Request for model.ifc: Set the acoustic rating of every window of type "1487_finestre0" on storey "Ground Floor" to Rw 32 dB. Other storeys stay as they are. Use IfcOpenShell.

First a look at what the model holds.

```python
import ifcopenshell
import ifcopenshell.util.element

model = ifcopenshell.open("model.ifc")
print(model.schema)
storey = next(s for s in model.by_type("IfcBuildingStorey") if s.Name == "Ground Floor")
windows = [e for e in ifcopenshell.util.element.get_decomposition(storey) if e.is_a("IfcWindow")]
seen = {}
for e in windows:
    element_type = ifcopenshell.util.element.get_type(e)
    key = (element_type.Name if element_type != e and element_type else None, ifcopenshell.util.element.get_pset(e, "Pset_WindowCommon", "AcousticRating"))
    seen[key] = seen.get(key, 0) + 1
for (name, value), count in sorted(seen.items(), key=str):
    print(count, "x", name, "|", value)
```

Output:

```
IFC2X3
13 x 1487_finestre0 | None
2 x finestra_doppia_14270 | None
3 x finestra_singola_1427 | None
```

```python
import ifcopenshell
import ifcopenshell.api.pset
import ifcopenshell.util.element

model = ifcopenshell.open("model.ifc")

storey = next(s for s in model.by_type("IfcBuildingStorey") if s.Name == "Ground Floor")
windows = [e for e in ifcopenshell.util.element.get_decomposition(storey) if e.is_a("IfcWindow")]

count = 0
for e in windows:
    element_type = ifcopenshell.util.element.get_type(e)
    if element_type in (None, e) or element_type.Name != "1487_finestre0":
        continue
    # add_pset returns the element's existing set when there is one.
    pset = ifcopenshell.api.pset.add_pset(model, product=e, name="Pset_WindowCommon")
    ifcopenshell.api.pset.edit_pset(model, pset=pset, properties={"AcousticRating": "Rw 32 dB"})
    count += 1

print(count, "windows updated")

model.write("model_updated.ifc")
```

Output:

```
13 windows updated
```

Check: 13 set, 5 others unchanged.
